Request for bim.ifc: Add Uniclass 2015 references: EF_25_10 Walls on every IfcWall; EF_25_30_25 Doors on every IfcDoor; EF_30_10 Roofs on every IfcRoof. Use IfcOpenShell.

First a look at what the model holds.

```python
import ifcopenshell

model = ifcopenshell.open("bim.ifc")
print(model.schema)
print("classifications:", [c.Name for c in model.by_type("IfcClassification")])
for ifc_class in ("IfcDoor", "IfcRoof", "IfcStair", "IfcWall", "IfcWindow"):
    print(ifc_class, len(model.by_type(ifc_class)))
```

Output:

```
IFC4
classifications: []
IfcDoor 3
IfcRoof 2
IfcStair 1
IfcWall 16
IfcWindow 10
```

```python
import ifcopenshell
import ifcopenshell.api.classification

model = ifcopenshell.open("bim.ifc")

system = ifcopenshell.api.classification.add_classification(model, classification="Uniclass 2015")

codes = {
    "IfcWall": ("EF_25_10", "Walls"),
    "IfcDoor": ("EF_25_30_25", "Doors"),
    "IfcRoof": ("EF_30_10", "Roofs"),
}
for ifc_class, (code, name) in codes.items():
    products = model.by_type(ifc_class)
    ifcopenshell.api.classification.add_reference(
        model, products=products, classification=system, identification=code, name=name
    )
    print(code, len(products))

model.write("bim_rev.ifc")
```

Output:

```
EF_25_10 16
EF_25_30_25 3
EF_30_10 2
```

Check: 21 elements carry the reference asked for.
